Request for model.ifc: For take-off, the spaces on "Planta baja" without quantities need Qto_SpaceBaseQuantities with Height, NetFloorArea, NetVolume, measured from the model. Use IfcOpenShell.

First a look at what the model holds.

```python
import ifcopenshell
import ifcopenshell.util.element
import ifcopenshell.util.unit

model = ifcopenshell.open("model.ifc")
print(model.schema)
for unit_type in ("LENGTHUNIT", "AREAUNIT", "VOLUMEUNIT"):
    print(unit_type, ifcopenshell.util.unit.calculate_unit_scale(model, unit_type))
storey = next(s for s in model.by_type("IfcBuildingStorey") if s.Name == "Planta baja")
spaces = [e for e in ifcopenshell.util.element.get_decomposition(storey) if e.is_a("IfcSpace")]
for e in sorted(spaces, key=lambda e: e.id()):
    print(e.id(), e.is_a(), e.Name, list(ifcopenshell.util.element.get_psets(e, qtos_only=True)), sep=" | ")
```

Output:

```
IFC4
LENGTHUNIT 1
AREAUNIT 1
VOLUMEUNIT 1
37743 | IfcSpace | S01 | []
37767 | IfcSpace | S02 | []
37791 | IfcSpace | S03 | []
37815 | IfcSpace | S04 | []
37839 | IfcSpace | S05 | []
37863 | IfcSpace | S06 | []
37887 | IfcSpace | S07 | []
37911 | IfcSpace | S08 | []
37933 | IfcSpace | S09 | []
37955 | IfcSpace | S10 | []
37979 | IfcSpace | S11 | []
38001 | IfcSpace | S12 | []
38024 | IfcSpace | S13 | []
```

```python
import ifcopenshell
import ifcopenshell.api.pset
import ifcopenshell.geom
import ifcopenshell.util.element
import ifcopenshell.util.shape
import ifcopenshell.util.unit

model = ifcopenshell.open("model.ifc")
unit_scale = ifcopenshell.util.unit.calculate_unit_scale(model)
area_scale = ifcopenshell.util.unit.calculate_unit_scale(model, "AREAUNIT")
volume_scale = ifcopenshell.util.unit.calculate_unit_scale(model, "VOLUMEUNIT")
settings = ifcopenshell.geom.settings()

storey = next(s for s in model.by_type("IfcBuildingStorey") if s.Name == "Planta baja")
spaces = [e for e in ifcopenshell.util.element.get_decomposition(storey) if e.is_a("IfcSpace")]

for e in sorted(spaces, key=lambda e: e.id()):
    if ifcopenshell.util.element.get_psets(e, qtos_only=True, should_inherit=False):
        continue
    # Geometry comes back in metres, in the element's own axes.
    shape = ifcopenshell.geom.create_shape(settings, e)
    values = {
        "Height": ifcopenshell.util.shape.get_z(shape.geometry) / unit_scale,
        "NetFloorArea": ifcopenshell.util.shape.get_footprint_area(shape.geometry) / area_scale,
        "NetVolume": ifcopenshell.util.shape.get_volume(shape.geometry) / volume_scale,
    }
    qto = ifcopenshell.api.pset.add_qto(model, product=e, name="Qto_SpaceBaseQuantities")
    ifcopenshell.api.pset.edit_qto(model, qto=qto, properties=values)
    print(e.id(), {k: round(v, 3) for k, v in values.items()})

model.write("model-out.ifc")
```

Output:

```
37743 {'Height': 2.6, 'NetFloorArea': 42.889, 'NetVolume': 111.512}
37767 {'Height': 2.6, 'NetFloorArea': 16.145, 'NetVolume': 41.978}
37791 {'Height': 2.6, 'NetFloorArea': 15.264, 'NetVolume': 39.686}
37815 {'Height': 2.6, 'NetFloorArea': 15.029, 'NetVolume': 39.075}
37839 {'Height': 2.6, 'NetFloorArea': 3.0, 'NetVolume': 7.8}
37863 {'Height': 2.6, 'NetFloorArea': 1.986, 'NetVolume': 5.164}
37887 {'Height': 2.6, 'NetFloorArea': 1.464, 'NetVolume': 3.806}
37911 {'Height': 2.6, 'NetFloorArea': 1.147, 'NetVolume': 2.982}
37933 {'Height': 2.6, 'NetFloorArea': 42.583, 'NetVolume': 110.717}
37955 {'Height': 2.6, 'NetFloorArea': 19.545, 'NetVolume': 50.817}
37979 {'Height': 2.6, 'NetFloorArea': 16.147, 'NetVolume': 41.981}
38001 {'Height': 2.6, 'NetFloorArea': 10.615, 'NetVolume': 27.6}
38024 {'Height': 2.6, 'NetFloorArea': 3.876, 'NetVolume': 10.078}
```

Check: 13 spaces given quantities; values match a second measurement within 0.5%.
